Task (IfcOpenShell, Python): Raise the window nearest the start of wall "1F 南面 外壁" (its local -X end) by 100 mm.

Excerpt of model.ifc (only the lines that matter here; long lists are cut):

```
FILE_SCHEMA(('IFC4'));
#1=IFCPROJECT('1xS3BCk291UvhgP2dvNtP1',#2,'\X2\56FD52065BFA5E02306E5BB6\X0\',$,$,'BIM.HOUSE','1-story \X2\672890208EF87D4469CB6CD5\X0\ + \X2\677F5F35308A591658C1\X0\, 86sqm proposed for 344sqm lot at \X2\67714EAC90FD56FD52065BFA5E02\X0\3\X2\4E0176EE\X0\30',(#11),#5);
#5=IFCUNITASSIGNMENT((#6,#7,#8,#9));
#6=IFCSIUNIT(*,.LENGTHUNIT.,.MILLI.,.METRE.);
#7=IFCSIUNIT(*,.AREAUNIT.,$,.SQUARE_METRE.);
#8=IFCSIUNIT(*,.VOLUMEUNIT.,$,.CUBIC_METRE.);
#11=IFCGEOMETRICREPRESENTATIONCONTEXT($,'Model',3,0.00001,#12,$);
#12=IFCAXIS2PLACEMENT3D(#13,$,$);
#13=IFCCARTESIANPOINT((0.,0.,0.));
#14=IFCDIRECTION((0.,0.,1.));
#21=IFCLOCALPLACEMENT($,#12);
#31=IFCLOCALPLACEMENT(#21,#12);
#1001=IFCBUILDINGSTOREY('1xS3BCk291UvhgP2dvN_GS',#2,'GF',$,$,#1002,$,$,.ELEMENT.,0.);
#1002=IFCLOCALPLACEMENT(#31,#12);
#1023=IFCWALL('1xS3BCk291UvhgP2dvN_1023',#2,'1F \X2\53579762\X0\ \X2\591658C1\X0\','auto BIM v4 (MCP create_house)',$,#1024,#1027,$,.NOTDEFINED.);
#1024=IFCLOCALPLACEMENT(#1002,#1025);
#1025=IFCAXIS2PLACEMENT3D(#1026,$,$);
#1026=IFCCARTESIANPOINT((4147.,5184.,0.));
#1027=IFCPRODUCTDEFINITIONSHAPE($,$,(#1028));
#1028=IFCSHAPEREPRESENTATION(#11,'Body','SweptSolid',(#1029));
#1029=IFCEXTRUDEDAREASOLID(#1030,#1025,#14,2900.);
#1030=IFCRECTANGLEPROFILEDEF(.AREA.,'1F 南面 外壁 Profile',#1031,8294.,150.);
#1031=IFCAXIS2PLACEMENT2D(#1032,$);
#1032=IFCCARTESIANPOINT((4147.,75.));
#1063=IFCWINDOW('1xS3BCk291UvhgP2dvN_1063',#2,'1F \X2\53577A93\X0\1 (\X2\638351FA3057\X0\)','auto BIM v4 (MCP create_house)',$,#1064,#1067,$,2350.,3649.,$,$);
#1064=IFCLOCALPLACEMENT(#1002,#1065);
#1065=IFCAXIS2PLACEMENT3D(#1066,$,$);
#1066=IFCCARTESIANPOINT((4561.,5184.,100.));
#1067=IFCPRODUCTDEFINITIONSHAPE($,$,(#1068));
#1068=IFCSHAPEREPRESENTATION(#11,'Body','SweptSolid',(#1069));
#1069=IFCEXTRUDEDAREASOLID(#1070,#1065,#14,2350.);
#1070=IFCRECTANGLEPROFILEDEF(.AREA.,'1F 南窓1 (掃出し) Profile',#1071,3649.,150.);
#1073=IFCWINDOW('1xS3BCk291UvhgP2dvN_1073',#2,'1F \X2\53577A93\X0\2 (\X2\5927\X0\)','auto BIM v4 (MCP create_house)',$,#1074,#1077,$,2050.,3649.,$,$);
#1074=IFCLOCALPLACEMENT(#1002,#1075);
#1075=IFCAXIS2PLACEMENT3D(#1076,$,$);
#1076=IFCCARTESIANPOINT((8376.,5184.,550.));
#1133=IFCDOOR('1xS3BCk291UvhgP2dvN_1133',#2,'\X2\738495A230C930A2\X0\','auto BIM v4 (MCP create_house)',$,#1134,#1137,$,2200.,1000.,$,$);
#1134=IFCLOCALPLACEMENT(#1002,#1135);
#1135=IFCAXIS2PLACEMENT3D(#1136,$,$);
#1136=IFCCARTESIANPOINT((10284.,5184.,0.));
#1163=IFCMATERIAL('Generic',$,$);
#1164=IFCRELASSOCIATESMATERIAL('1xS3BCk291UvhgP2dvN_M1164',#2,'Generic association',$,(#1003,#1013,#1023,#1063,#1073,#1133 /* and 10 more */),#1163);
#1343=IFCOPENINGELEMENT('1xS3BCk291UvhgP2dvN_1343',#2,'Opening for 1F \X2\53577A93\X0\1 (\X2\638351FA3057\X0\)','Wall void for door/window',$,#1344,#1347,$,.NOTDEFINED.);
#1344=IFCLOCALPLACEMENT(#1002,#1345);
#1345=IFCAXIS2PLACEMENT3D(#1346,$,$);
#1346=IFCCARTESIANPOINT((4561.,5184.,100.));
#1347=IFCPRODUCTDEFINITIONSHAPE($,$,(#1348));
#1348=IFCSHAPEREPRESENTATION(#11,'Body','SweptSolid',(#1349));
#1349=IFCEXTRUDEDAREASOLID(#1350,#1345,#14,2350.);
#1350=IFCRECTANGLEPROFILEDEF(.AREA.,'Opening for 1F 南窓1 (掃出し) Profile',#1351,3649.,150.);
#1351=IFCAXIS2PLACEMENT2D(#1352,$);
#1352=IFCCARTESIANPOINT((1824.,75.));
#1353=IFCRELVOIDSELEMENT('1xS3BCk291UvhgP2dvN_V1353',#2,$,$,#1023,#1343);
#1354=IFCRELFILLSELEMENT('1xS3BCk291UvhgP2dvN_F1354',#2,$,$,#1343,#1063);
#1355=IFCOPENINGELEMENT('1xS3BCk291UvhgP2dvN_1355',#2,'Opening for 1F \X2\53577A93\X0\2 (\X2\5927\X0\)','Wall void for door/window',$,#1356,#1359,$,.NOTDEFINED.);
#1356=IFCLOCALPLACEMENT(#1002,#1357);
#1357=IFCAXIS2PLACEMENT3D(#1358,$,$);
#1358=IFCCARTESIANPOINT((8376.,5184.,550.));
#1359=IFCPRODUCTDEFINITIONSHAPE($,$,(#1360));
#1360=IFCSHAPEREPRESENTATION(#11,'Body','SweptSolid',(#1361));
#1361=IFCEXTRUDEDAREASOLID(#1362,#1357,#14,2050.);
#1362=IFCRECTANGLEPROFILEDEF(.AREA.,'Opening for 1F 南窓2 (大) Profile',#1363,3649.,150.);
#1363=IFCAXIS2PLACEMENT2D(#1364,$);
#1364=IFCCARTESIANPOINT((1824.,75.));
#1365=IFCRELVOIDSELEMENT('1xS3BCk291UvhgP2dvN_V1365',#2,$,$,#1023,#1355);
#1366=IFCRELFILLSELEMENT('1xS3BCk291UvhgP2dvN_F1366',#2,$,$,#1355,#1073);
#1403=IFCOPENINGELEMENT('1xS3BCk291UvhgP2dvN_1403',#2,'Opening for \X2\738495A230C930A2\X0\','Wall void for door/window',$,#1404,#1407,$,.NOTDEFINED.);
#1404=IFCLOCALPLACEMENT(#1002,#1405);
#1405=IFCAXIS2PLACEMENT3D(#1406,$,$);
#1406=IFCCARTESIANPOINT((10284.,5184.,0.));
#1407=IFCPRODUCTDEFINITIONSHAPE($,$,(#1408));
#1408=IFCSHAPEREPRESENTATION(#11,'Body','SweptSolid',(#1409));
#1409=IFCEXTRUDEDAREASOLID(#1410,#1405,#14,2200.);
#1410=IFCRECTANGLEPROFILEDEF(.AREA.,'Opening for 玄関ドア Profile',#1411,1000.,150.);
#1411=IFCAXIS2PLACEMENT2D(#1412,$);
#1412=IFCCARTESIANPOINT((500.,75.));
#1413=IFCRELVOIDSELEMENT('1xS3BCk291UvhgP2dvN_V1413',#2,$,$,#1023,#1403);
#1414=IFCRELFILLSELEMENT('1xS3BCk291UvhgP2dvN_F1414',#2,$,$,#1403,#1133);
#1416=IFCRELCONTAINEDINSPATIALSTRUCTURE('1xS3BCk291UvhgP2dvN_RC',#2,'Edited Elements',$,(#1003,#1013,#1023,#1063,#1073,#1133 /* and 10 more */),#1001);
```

```python
import numpy as np
import ifcopenshell
import ifcopenshell.api.geometry
import ifcopenshell.util.placement
import ifcopenshell.util.unit

model = ifcopenshell.open("model.ifc")
unit_scale = ifcopenshell.util.unit.calculate_unit_scale(model)

window = model.by_guid("1xS3BCk291UvhgP2dvN_1063")
opening = window.FillsVoids[0].RelatingOpeningElement
dz = 0.1 / unit_scale

shift = np.array([0.0, 0.0, dz])
# The window is not placed relative to its opening, so move both.
for product in (opening, window):
    matrix = ifcopenshell.util.placement.get_local_placement(product.ObjectPlacement)
    matrix[:3, 3] += shift
    ifcopenshell.api.geometry.edit_object_placement(model, product=product, matrix=matrix, is_si=False)

print(f"moved by {dz * unit_scale:+.3f} m")

model.write("model_rev.ifc")
```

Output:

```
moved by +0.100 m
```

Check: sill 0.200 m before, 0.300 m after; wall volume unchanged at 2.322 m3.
